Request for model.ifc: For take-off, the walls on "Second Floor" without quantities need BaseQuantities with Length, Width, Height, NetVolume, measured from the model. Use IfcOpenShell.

First a look at what the model holds.

```python
import ifcopenshell
import ifcopenshell.util.element
import ifcopenshell.util.unit

model = ifcopenshell.open("model.ifc")
print(model.schema)
for unit_type in ("LENGTHUNIT", "AREAUNIT", "VOLUMEUNIT"):
    print(unit_type, ifcopenshell.util.unit.calculate_unit_scale(model, unit_type))
storey = next(s for s in model.by_type("IfcBuildingStorey") if s.Name == "Second Floor")
walls = [e for e in ifcopenshell.util.element.get_decomposition(storey) if e.is_a("IfcWall")]
for e in sorted(walls, key=lambda e: e.id()):
    print(e.id(), e.is_a(), e.Name, list(ifcopenshell.util.element.get_psets(e, qtos_only=True)), sep=" | ")
```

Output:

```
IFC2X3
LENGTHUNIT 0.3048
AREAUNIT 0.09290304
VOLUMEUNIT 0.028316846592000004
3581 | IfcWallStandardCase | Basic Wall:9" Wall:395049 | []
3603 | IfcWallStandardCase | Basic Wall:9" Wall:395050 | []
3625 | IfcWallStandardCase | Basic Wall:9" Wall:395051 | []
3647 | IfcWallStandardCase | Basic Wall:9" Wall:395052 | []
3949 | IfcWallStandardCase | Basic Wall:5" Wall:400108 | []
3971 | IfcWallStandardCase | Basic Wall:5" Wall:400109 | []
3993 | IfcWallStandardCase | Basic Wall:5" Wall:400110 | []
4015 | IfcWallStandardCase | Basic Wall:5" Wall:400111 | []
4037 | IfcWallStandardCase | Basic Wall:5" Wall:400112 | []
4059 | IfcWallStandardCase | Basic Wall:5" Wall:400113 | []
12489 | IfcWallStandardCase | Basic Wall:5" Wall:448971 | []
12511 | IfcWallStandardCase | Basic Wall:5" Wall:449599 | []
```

```python
import ifcopenshell
import ifcopenshell.api.pset
import ifcopenshell.geom
import ifcopenshell.util.element
import ifcopenshell.util.shape
import ifcopenshell.util.unit

model = ifcopenshell.open("model.ifc")
unit_scale = ifcopenshell.util.unit.calculate_unit_scale(model)
volume_scale = ifcopenshell.util.unit.calculate_unit_scale(model, "VOLUMEUNIT")
settings = ifcopenshell.geom.settings()

storey = next(s for s in model.by_type("IfcBuildingStorey") if s.Name == "Second Floor")
walls = [e for e in ifcopenshell.util.element.get_decomposition(storey) if e.is_a("IfcWall")]

for e in sorted(walls, key=lambda e: e.id()):
    if ifcopenshell.util.element.get_psets(e, qtos_only=True, should_inherit=False):
        continue
    # Geometry comes back in metres, in the element's own axes.
    shape = ifcopenshell.geom.create_shape(settings, e)
    values = {
        "Length": ifcopenshell.util.shape.get_x(shape.geometry) / unit_scale,
        "Width": ifcopenshell.util.shape.get_y(shape.geometry) / unit_scale,
        "Height": ifcopenshell.util.shape.get_z(shape.geometry) / unit_scale,
        "NetVolume": ifcopenshell.util.shape.get_volume(shape.geometry) / volume_scale,
    }
    qto = ifcopenshell.api.pset.add_qto(model, product=e, name="BaseQuantities")
    ifcopenshell.api.pset.edit_qto(model, qto=qto, properties=values)
    print(e.id(), {k: round(v, 3) for k, v in values.items()})

model.write("model-out.ifc")
```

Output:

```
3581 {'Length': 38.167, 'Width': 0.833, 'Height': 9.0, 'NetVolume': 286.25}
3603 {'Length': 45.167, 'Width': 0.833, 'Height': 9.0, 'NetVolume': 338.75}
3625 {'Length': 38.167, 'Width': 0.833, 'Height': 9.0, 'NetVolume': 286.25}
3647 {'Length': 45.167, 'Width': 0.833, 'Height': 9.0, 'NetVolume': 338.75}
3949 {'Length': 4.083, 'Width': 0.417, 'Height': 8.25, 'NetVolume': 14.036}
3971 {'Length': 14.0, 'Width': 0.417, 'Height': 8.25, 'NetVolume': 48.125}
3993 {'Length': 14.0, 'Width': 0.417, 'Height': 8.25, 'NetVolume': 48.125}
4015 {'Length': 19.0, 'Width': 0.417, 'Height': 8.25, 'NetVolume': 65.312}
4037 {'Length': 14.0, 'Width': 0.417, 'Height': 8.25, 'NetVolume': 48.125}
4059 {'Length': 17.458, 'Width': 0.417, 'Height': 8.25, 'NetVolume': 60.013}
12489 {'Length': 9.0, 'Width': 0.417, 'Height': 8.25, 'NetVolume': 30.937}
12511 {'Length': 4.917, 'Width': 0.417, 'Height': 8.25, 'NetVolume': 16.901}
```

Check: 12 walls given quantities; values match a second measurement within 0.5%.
